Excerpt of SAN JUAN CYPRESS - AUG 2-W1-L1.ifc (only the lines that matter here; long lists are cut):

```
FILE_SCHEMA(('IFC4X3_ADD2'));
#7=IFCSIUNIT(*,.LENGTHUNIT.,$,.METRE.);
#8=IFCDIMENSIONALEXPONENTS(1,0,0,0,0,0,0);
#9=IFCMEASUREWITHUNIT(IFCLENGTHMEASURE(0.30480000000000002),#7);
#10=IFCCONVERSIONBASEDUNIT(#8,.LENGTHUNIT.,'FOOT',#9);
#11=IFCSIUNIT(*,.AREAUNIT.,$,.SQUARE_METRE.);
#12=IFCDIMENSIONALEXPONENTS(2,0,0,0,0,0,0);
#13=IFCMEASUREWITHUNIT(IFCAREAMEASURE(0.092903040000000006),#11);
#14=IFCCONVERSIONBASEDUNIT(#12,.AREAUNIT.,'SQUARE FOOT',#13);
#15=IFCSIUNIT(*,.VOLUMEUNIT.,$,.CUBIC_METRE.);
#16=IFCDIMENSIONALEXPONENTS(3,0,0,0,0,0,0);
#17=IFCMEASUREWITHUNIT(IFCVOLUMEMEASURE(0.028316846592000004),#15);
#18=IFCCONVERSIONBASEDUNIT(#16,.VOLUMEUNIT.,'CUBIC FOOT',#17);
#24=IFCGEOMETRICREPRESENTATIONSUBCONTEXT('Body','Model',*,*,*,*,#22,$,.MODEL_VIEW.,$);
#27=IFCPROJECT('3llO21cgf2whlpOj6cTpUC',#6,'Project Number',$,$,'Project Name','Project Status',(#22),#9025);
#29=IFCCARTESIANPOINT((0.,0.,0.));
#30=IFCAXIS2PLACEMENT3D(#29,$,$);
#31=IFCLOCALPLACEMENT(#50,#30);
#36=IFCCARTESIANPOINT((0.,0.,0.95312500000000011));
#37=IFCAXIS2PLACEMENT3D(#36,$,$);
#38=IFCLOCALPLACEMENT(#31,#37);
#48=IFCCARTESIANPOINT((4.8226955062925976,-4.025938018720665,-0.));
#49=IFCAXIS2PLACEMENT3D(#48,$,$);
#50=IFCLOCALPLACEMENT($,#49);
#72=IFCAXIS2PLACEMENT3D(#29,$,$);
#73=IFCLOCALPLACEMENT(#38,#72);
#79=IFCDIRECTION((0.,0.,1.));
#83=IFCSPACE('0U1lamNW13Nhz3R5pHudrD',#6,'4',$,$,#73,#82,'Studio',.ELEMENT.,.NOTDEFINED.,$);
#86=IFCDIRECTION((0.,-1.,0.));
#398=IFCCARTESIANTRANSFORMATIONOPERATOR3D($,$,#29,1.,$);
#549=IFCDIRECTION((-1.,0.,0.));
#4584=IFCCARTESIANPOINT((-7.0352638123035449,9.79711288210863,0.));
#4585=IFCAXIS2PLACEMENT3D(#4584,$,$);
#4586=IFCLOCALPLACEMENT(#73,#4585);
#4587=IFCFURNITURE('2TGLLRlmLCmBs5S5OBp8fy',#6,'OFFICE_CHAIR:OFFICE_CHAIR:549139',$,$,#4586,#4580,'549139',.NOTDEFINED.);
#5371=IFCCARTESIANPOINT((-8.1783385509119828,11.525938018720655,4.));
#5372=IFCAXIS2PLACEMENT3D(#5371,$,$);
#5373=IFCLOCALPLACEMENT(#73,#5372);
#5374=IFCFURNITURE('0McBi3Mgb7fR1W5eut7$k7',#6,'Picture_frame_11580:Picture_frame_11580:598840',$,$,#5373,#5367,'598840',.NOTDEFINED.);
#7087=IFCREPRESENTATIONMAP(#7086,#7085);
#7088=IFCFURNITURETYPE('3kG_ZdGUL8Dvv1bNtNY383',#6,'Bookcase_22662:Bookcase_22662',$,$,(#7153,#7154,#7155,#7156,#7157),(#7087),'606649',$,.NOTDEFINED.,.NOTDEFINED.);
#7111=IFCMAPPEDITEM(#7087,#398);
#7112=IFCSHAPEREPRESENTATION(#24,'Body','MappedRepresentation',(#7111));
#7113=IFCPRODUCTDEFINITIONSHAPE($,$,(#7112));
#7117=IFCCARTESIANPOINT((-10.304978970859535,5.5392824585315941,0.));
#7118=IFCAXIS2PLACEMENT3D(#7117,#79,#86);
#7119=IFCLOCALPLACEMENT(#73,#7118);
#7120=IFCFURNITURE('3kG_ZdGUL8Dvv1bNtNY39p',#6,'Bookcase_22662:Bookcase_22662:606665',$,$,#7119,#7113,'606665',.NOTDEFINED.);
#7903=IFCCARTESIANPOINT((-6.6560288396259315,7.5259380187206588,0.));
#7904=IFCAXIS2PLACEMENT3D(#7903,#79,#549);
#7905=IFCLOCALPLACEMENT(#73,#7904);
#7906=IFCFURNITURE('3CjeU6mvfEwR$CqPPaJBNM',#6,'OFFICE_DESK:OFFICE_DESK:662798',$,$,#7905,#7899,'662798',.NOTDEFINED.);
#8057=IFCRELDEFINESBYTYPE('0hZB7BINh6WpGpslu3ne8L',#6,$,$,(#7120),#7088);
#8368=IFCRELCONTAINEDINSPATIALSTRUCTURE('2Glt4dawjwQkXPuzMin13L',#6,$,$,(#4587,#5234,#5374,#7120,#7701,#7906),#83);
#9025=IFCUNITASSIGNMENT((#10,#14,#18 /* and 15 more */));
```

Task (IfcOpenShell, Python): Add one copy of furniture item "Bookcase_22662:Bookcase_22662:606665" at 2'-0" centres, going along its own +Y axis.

```python
import ifcopenshell
import ifcopenshell.api.geometry
import ifcopenshell.api.root
import ifcopenshell.util.element
import ifcopenshell.util.placement
import ifcopenshell.util.unit

model = ifcopenshell.open("SAN JUAN CYPRESS - AUG 2-W1-L1.ifc")
unit_scale = ifcopenshell.util.unit.calculate_unit_scale(model)


def reuse_history(source, copy):
    """copy_class also copies each property set's owner history, people and application; keep the originals."""
    for rel in copy.IsDefinedBy:
        if rel.is_a("IfcRelDefinesByProperties") and (history := rel.RelatingPropertyDefinition.OwnerHistory):
            rel.RelatingPropertyDefinition.OwnerHistory = source.OwnerHistory
            ifcopenshell.util.element.remove_deep2(model, history)


source = model.by_guid("3kG_ZdGUL8Dvv1bNtNY39p")
base = ifcopenshell.util.placement.get_local_placement(source.ObjectPlacement)
step = base[:3, 1] * 24 * 0.0254 / unit_scale

for i in range(1, 2):
    copy = ifcopenshell.api.root.copy_class(model, product=source)
    copy.Representation = ifcopenshell.util.element.copy_deep(
        model, source.Representation, exclude=["IfcGeometricRepresentationContext", "IfcRepresentationMap"]
    )
    copy.Name = "Bookcase_22662:Bookcase_22662"
    copy.Tag = None
    reuse_history(source, copy)
    matrix = base.copy()
    matrix[:3, 3] += i * step
    print("added at", matrix[:3, 3].round(3) + 0.0)
    ifcopenshell.api.geometry.edit_object_placement(model, product=copy, matrix=matrix, is_si=False)

model.write("SAN JUAN CYPRESS - AUG 2-W1-L1_rev.ifc")
```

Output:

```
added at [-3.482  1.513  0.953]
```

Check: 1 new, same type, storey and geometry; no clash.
